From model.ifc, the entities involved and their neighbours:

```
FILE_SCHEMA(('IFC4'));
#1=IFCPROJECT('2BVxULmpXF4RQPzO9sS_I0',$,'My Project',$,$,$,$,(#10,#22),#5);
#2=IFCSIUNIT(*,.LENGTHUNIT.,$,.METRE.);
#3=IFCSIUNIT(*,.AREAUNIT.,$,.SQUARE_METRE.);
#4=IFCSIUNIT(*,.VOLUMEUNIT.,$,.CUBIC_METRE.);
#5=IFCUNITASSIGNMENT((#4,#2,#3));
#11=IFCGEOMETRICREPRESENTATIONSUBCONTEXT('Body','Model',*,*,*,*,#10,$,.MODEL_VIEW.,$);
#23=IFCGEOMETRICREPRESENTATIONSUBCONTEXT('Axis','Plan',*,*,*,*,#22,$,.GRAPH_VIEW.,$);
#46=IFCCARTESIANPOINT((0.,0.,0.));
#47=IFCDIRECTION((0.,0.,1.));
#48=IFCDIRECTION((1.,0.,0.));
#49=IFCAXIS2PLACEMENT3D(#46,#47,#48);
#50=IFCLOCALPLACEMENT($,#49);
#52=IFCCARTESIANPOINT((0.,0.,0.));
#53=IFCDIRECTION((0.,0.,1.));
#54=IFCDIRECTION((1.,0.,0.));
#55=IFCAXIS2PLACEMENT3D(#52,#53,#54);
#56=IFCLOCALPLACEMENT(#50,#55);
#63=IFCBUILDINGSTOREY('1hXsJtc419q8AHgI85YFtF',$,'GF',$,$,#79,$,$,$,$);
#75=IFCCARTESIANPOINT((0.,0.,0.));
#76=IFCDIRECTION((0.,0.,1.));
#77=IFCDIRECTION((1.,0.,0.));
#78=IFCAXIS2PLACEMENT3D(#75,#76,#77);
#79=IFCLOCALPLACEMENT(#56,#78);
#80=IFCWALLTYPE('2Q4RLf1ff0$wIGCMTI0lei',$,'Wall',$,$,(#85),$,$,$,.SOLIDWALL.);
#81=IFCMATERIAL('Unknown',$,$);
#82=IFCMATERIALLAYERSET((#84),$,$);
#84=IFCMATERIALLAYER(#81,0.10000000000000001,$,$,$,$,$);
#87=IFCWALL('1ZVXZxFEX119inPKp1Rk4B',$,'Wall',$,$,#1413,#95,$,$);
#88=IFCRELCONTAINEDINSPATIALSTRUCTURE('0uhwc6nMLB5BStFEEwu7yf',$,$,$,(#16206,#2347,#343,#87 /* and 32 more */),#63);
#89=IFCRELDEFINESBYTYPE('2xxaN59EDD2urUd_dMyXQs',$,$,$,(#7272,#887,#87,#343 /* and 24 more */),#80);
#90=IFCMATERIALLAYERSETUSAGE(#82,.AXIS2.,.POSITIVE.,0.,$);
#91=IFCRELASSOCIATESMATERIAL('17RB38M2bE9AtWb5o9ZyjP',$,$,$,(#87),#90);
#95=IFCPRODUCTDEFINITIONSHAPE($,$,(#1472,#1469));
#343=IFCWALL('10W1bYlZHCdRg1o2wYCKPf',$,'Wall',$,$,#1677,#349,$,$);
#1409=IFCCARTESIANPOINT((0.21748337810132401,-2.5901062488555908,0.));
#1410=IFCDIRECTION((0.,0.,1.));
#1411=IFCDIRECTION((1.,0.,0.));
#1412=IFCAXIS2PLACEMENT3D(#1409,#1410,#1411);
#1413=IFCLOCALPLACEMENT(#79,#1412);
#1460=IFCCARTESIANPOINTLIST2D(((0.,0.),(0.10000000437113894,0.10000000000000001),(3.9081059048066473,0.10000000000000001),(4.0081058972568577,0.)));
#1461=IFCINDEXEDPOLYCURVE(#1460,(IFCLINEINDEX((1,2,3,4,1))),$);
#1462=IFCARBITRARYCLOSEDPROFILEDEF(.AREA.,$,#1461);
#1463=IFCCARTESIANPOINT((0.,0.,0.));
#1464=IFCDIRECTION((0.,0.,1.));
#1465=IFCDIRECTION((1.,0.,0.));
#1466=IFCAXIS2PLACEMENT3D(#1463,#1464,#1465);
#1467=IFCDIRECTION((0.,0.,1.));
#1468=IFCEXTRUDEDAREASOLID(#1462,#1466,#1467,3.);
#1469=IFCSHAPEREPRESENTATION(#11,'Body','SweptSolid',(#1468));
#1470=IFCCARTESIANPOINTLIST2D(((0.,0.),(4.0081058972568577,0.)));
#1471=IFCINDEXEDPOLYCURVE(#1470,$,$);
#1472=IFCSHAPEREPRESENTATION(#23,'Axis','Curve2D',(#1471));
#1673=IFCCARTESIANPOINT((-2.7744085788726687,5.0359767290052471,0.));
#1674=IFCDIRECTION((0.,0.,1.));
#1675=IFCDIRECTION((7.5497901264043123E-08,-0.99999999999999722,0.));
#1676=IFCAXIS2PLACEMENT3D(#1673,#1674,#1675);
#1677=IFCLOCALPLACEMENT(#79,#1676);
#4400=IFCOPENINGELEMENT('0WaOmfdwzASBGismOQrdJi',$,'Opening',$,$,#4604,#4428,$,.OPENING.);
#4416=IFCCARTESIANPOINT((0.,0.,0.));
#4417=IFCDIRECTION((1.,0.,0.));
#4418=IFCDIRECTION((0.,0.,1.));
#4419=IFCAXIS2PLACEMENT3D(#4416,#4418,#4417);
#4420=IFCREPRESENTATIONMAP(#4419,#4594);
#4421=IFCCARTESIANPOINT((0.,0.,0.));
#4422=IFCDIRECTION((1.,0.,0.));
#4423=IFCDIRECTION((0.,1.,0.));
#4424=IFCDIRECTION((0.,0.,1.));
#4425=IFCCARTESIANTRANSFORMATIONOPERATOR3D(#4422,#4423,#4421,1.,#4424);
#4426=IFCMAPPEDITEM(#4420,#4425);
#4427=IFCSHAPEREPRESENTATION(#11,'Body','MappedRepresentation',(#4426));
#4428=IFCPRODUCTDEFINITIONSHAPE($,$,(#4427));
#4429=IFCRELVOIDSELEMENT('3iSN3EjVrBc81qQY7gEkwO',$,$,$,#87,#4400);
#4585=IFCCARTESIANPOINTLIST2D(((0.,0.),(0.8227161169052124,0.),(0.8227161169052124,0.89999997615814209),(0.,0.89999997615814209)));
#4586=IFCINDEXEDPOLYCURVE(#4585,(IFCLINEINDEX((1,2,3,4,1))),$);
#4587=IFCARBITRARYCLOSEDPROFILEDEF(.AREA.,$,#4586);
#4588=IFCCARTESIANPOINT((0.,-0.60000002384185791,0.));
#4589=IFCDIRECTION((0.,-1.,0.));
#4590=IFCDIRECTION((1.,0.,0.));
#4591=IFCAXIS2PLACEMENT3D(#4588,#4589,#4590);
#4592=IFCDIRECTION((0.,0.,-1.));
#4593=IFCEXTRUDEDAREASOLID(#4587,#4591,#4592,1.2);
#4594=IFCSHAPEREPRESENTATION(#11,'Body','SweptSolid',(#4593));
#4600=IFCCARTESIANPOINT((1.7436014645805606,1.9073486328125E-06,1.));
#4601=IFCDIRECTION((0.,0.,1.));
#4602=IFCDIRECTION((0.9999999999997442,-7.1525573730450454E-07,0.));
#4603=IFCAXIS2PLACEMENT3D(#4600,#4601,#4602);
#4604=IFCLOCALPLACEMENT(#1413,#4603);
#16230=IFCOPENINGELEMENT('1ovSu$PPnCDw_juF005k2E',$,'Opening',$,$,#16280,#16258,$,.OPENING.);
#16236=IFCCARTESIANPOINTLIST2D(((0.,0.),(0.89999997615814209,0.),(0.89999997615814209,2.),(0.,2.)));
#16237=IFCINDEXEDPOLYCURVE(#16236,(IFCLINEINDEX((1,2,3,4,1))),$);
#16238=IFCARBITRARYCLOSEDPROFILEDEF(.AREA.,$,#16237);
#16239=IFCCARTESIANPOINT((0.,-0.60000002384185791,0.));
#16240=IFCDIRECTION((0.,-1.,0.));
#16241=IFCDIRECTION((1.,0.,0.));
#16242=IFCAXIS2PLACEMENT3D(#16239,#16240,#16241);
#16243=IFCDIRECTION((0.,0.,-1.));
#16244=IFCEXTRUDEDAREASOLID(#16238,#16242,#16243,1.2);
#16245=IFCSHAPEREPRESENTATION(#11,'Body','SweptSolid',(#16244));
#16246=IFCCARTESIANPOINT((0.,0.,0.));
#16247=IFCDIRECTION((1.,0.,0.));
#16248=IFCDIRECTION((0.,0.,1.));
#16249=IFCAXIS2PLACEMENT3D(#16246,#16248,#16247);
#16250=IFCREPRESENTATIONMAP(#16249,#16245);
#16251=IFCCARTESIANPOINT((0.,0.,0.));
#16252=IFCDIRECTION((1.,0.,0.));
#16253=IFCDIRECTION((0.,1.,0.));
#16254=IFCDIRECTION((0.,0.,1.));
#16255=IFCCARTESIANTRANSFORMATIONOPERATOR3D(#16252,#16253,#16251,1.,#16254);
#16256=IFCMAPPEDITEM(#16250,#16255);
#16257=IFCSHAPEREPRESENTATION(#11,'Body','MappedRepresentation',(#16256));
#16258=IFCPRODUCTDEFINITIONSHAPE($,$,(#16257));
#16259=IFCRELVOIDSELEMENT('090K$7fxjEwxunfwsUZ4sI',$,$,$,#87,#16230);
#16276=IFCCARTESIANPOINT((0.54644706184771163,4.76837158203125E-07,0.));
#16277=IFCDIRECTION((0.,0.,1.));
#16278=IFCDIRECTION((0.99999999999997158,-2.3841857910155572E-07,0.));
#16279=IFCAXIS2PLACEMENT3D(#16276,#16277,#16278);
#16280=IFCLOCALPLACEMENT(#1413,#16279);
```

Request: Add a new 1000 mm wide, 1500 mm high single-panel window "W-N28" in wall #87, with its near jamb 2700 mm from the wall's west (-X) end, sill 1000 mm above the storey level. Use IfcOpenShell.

```python
import numpy as np
import ifcopenshell
import ifcopenshell.api.feature
import ifcopenshell.api.geometry
import ifcopenshell.api.root
import ifcopenshell.api.spatial
import ifcopenshell.geom
import ifcopenshell.util.element
import ifcopenshell.util.placement
import ifcopenshell.util.representation
import ifcopenshell.util.shape
import ifcopenshell.util.unit

model = ifcopenshell.open("model.ifc")
unit_scale = ifcopenshell.util.unit.calculate_unit_scale(model)
settings = ifcopenshell.geom.settings()


def volume(element):
    """Net volume in cubic metres, openings subtracted."""
    shape = ifcopenshell.geom.create_shape(settings, element)
    return ifcopenshell.util.shape.get_volume(shape.geometry)


wall = model.by_id(87)
storey = ifcopenshell.util.element.get_container(wall, ifc_class="IfcBuildingStorey")
context = ifcopenshell.util.representation.get_context(model, "Model", "Body", "MODEL_VIEW")
before = volume(wall)

width, height, from_end, sill = 1, 1.5, 2.7, 1  # metres

# The wall runs along its own X axis, and the end named is its -X end.
wall_shape = ifcopenshell.geom.create_shape(settings, wall)
x, y, z = ifcopenshell.util.shape.get_vertices(wall_shape.geometry).T
start = x.min() + from_end
face, thickness = float(y.min()), float(y.max() - y.min())
wall_matrix = ifcopenshell.util.placement.get_local_placement(wall.ObjectPlacement)
level = ifcopenshell.util.placement.get_local_placement(storey.ObjectPlacement)[2, 3]


def in_wall(x, y):
    """Placement at x, y metres in the wall's axes, at sill height."""
    matrix = wall_matrix.copy()
    matrix[:, 3] = wall_matrix @ np.array([x / unit_scale, y / unit_scale, 0.0, 1.0])
    matrix[2, 3] = level + sill / unit_scale
    return matrix


# Opening: a box that overshoots both wall faces by 50 mm.
opening = ifcopenshell.api.root.create_entity(model, ifc_class="IfcOpeningElement", predefined_type="OPENING")
box = ifcopenshell.api.geometry.add_wall_representation(
    model, context=context, length=width, height=height, thickness=thickness + 0.1
)
ifcopenshell.api.geometry.assign_representation(model, product=opening, representation=box)
ifcopenshell.api.geometry.edit_object_placement(model, product=opening, matrix=in_wall(start, face - 0.05), is_si=False)
ifcopenshell.api.feature.add_feature(model, feature=opening, element=wall)

window = ifcopenshell.api.root.create_entity(model, ifc_class="IfcWindow", name="W-N28", predefined_type="WINDOW")
window.OverallWidth, window.OverallHeight = width / unit_scale, height / unit_scale
window.PartitioningType = "SINGLE_PANEL"
body = ifcopenshell.api.geometry.add_window_representation(
    model,
    context=context,
    overall_width=window.OverallWidth,
    overall_height=window.OverallHeight,
    partition_type="SINGLE_PANEL",
)
ifcopenshell.api.geometry.assign_representation(model, product=window, representation=body)
ifcopenshell.api.spatial.assign_container(model, products=[window], relating_structure=storey)
ifcopenshell.api.feature.add_filling(model, opening=opening, element=window)

# Centre the window in the wall's thickness.
ifcopenshell.api.geometry.edit_object_placement(model, product=window, matrix=in_wall(start, face), is_si=False)
window_shape = ifcopenshell.geom.create_shape(settings, window)
depth = ifcopenshell.util.shape.get_vertices(window_shape.geometry)[:, 1]
offset = face + thickness / 2 - (depth.min() + depth.max()) / 2
ifcopenshell.api.geometry.edit_object_placement(model, product=window, matrix=in_wall(start, offset), is_si=False)

after = volume(wall)

print(f"wall volume {before:.3f} -> {after:.3f} m3")

model.write("model_v2.ifc")
```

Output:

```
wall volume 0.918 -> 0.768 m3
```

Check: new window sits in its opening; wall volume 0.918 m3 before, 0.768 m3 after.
